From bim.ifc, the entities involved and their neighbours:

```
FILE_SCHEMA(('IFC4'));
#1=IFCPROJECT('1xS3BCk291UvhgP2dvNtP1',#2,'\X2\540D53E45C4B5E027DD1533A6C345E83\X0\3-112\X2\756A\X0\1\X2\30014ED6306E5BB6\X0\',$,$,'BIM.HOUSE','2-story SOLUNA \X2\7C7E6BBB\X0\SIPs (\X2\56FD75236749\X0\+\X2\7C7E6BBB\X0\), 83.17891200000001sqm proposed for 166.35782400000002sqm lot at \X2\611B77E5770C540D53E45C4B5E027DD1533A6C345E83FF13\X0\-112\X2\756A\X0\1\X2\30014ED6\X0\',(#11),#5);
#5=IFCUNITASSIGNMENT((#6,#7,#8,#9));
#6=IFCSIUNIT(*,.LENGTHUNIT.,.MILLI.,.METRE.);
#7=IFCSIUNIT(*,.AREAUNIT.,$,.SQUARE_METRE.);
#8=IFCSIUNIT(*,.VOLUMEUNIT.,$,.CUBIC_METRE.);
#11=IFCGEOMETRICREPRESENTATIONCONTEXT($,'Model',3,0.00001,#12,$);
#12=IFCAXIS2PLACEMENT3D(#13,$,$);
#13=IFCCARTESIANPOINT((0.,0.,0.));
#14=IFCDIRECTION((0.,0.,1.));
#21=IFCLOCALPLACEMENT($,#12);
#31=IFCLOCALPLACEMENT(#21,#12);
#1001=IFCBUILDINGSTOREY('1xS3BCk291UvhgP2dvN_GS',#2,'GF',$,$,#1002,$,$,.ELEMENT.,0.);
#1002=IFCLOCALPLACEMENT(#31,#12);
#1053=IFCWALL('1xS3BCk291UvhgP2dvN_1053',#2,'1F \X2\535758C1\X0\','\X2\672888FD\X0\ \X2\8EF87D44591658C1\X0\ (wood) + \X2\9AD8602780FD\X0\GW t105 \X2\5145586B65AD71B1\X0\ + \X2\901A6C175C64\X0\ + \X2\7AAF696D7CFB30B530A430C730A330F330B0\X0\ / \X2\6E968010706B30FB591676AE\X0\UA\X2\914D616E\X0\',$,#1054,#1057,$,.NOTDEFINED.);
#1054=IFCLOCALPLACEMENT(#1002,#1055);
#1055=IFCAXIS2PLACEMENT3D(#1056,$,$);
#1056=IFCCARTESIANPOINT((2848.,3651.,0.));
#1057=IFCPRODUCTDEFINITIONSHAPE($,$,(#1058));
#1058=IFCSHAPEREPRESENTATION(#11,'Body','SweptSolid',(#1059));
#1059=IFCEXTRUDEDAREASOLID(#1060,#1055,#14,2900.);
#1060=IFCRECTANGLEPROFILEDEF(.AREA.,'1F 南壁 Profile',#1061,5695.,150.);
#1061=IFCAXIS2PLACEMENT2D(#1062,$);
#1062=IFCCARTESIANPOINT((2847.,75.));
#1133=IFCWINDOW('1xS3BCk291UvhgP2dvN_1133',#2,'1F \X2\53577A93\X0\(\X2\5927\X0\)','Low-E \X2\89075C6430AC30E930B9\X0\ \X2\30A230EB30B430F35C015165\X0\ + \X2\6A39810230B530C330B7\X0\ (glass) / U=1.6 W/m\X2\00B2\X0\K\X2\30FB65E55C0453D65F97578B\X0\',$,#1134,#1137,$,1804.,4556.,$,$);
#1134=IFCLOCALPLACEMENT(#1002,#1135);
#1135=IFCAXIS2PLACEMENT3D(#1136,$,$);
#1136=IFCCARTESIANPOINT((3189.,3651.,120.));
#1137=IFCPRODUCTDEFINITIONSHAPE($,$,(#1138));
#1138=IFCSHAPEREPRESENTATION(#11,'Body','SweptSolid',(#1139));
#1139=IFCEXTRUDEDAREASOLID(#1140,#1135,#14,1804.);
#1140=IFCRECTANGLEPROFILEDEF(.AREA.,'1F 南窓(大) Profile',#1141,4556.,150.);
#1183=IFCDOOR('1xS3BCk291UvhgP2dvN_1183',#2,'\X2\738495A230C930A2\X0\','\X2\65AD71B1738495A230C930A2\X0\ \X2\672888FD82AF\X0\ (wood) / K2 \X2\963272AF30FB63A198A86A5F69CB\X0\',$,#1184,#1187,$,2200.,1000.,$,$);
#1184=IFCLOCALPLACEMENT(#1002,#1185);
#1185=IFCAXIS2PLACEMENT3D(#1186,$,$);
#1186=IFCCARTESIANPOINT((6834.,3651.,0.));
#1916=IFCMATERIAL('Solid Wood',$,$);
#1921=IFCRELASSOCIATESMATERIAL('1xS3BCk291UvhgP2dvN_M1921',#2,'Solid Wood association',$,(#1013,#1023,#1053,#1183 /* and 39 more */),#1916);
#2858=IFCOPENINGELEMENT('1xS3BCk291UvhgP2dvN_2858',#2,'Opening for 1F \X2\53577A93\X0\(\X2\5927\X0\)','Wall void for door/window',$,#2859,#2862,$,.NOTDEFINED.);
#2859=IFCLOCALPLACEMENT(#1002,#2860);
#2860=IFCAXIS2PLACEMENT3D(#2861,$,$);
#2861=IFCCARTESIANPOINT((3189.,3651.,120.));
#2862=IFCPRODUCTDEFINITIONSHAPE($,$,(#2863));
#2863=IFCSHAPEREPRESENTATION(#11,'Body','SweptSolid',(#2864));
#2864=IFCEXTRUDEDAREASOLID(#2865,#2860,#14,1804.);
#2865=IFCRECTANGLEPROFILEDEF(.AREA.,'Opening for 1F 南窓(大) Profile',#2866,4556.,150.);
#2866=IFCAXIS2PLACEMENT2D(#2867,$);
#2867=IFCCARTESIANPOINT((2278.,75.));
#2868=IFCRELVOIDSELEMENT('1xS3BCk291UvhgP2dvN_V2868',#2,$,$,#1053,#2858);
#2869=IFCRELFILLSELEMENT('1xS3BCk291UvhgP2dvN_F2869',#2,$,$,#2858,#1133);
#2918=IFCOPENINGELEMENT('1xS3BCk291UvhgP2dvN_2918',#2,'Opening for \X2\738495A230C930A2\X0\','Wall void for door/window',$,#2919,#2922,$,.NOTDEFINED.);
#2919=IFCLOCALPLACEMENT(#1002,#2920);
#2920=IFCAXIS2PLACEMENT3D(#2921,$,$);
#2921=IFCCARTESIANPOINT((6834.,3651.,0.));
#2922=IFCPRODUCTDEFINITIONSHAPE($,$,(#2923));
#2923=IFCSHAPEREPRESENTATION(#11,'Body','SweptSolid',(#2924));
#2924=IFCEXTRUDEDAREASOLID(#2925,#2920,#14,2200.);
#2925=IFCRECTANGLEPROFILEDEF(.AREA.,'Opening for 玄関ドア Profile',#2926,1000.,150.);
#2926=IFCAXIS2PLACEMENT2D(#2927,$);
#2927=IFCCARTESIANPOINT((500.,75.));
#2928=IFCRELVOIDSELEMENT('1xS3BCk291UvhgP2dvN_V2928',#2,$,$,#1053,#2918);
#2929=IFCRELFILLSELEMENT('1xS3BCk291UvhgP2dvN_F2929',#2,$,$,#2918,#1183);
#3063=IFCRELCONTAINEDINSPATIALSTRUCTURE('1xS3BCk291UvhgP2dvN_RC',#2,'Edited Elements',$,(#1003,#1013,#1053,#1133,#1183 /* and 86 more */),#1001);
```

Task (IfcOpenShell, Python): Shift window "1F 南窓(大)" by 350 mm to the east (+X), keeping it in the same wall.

```python
import ifcopenshell
import ifcopenshell.api.geometry
import ifcopenshell.util.placement

model = ifcopenshell.open("bim.ifc")

window = model.by_id(1133)
opening = window.FillsVoids[0].RelatingOpeningElement
wall = opening.VoidsElements[0].RelatingBuildingElement

wall_matrix = ifcopenshell.util.placement.get_local_placement(wall.ObjectPlacement)
shift = wall_matrix[:3, 0] * 350.0
before = ifcopenshell.util.placement.get_local_placement(window.ObjectPlacement)[:3, 3].copy()

# The window is not placed relative to its opening, so move both.
for product in (opening, window):
    matrix = ifcopenshell.util.placement.get_local_placement(product.ObjectPlacement)
    matrix[:3, 3] += shift
    ifcopenshell.api.geometry.edit_object_placement(model, product=product, matrix=matrix, is_si=False)

after = ifcopenshell.util.placement.get_local_placement(window.ObjectPlacement)[:3, 3]
print("window moved by", (after - before).round(3) + 0.0)

model.write("bim-out.ifc")
```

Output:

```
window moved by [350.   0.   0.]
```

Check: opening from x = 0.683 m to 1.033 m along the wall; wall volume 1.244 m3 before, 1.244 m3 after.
